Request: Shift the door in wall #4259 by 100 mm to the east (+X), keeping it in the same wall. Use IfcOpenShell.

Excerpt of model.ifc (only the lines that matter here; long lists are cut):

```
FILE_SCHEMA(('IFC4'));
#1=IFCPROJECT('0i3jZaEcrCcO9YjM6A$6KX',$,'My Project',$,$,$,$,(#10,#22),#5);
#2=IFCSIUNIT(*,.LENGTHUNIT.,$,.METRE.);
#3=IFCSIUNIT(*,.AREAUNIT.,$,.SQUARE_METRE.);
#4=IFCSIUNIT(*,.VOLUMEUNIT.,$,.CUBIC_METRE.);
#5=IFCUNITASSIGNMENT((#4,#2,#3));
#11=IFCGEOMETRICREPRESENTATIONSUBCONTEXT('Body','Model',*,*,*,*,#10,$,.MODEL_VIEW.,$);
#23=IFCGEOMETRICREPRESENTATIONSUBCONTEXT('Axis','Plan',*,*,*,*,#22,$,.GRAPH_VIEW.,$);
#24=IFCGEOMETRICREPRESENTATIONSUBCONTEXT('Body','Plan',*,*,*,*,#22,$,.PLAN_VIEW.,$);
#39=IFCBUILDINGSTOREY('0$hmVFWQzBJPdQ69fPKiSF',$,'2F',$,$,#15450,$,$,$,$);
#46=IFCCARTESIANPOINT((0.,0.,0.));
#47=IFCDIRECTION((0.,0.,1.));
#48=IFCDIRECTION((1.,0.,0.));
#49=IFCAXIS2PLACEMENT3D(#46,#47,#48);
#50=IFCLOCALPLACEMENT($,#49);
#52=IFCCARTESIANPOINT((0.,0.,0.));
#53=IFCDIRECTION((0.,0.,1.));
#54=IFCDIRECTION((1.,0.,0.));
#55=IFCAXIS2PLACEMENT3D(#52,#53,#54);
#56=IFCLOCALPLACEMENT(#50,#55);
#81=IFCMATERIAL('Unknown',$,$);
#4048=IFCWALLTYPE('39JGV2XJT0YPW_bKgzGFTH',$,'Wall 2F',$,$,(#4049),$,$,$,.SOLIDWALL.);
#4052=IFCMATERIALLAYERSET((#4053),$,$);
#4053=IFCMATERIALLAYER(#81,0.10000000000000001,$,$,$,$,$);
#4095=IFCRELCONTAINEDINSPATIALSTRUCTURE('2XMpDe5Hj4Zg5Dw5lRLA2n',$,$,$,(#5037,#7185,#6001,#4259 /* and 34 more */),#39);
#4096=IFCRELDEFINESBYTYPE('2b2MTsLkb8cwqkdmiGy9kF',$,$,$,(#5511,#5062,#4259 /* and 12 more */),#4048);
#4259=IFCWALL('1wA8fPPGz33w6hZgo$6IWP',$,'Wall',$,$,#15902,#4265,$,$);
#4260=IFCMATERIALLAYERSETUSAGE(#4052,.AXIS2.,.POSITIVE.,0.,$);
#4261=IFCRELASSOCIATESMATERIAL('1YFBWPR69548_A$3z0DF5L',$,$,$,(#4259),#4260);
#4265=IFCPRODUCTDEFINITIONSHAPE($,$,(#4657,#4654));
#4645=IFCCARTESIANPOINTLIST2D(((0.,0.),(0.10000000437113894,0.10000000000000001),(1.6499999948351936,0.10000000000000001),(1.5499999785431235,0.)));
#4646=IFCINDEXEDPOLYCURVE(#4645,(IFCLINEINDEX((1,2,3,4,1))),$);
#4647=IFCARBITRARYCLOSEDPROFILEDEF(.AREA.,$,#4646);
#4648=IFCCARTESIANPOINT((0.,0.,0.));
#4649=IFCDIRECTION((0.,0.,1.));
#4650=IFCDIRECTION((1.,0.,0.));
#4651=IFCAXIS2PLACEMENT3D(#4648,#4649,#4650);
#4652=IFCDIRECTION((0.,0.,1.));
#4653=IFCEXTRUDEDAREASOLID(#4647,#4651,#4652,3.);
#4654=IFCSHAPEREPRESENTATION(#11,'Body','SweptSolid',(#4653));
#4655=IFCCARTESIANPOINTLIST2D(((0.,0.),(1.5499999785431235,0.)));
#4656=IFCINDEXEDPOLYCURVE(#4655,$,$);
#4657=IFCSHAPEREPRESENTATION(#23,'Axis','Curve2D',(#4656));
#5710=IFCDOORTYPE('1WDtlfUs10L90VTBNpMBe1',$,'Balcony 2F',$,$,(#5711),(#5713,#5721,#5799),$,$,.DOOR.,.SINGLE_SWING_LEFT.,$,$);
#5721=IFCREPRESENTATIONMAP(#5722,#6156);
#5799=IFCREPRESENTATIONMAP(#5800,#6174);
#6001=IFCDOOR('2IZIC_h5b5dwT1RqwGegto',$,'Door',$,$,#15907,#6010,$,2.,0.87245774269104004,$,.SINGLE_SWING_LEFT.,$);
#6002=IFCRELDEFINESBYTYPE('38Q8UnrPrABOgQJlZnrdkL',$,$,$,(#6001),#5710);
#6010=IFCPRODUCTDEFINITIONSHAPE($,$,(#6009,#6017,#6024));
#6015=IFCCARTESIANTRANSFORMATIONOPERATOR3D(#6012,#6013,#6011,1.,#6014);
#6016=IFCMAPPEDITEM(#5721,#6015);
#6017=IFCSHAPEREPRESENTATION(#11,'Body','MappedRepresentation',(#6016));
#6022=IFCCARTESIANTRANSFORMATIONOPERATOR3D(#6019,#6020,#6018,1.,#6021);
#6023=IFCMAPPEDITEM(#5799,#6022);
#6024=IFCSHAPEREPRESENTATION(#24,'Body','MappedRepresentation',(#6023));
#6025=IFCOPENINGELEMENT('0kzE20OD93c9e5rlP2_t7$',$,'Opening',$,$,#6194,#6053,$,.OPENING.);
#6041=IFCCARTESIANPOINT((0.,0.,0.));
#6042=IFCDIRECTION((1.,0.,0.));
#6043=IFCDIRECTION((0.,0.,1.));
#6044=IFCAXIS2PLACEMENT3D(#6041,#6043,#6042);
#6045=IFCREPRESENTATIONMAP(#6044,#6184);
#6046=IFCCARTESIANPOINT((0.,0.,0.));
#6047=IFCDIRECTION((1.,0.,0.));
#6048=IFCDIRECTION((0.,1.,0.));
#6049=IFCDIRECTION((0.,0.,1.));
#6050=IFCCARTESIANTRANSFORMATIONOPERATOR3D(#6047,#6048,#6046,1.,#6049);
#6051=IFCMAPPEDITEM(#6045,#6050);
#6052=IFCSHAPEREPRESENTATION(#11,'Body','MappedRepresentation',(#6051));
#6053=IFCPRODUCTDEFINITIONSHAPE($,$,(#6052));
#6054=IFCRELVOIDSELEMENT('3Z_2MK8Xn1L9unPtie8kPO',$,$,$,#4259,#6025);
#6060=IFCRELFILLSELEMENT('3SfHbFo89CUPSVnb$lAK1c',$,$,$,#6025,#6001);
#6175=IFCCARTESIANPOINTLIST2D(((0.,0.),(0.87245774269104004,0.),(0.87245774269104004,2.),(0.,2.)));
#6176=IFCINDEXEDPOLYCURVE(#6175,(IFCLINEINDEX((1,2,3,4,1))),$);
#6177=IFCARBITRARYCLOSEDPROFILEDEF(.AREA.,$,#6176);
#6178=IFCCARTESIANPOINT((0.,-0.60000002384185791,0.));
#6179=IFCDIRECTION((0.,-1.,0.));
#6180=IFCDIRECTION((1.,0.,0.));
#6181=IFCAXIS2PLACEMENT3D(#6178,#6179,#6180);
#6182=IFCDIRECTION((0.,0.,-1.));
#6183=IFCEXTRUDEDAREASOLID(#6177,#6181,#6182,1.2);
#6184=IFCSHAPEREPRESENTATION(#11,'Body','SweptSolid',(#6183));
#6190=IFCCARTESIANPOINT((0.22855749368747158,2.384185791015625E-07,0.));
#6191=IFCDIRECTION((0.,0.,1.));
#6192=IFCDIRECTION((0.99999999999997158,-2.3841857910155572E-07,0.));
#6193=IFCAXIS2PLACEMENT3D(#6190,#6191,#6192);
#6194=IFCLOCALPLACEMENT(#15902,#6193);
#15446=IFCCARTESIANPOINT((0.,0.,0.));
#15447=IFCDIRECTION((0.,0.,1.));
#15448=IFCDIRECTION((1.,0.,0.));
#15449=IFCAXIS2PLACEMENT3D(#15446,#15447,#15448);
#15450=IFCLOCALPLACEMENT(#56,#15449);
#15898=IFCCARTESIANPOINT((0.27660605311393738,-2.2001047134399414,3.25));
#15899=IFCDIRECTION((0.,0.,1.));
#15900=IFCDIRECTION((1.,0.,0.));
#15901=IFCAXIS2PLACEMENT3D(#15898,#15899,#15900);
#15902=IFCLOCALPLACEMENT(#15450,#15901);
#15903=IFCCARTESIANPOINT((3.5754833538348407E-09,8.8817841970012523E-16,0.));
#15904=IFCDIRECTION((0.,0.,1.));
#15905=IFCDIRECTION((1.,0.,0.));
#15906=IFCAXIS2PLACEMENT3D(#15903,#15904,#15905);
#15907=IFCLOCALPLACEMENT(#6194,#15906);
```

```python
import ifcopenshell
import ifcopenshell.api.geometry
import ifcopenshell.util.placement
import ifcopenshell.util.unit

model = ifcopenshell.open("model.ifc")
unit_scale = ifcopenshell.util.unit.calculate_unit_scale(model)

door = model.by_id(6001)
opening = door.FillsVoids[0].RelatingOpeningElement
wall = opening.VoidsElements[0].RelatingBuildingElement

wall_matrix = ifcopenshell.util.placement.get_local_placement(wall.ObjectPlacement)
shift = wall_matrix[:3, 0] * 0.1 / unit_scale
before = ifcopenshell.util.placement.get_local_placement(door.ObjectPlacement)[:3, 3].copy()

# The door is placed relative to its opening, so it follows when the opening moves.
matrix = ifcopenshell.util.placement.get_local_placement(opening.ObjectPlacement)
matrix[:3, 3] += shift
ifcopenshell.api.geometry.edit_object_placement(
    model, product=opening, matrix=matrix, is_si=False, should_transform_children=True
)

after = ifcopenshell.util.placement.get_local_placement(door.ObjectPlacement)[:3, 3]
print("door moved by", (after - before).round(3) + 0.0)

model.write("model_v2.ifc")
```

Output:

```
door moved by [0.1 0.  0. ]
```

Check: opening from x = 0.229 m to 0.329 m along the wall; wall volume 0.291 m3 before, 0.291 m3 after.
